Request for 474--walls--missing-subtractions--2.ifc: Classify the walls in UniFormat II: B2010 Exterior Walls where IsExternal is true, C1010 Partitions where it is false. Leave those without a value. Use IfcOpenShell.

First a look at what the model holds.

```python
import ifcopenshell
import ifcopenshell.util.element

model = ifcopenshell.open("474--walls--missing-subtractions--2.ifc")
print(model.schema)
print("classifications:", [c.Name for c in model.by_type("IfcClassification")])
values = [ifcopenshell.util.element.get_pset(e, "Pset_WallCommon", "IsExternal") for e in model.by_type("IfcWall")]
for value in (True, False, None):
    print("IsExternal", value, values.count(value))
```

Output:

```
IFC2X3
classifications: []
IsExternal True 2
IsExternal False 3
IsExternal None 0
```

```python
import ifcopenshell
import ifcopenshell.api.classification
import ifcopenshell.util.element

model = ifcopenshell.open("474--walls--missing-subtractions--2.ifc")

# IFC2X3 requires Source and Edition and has no link from the project to the system.
system = model.create_entity("IfcClassification", Source="ASTM", Edition="E1557", Name="UniFormat II")

walls = model.by_type("IfcWall")
external = {e: ifcopenshell.util.element.get_pset(e, "Pset_WallCommon", "IsExternal") for e in walls}
for flag, code, name in ((True, "B2010", "Exterior Walls"), (False, "C1010", "Partitions")):
    products = [e for e in walls if external[e] is flag]
    ifcopenshell.api.classification.add_reference(
        model, products=products, classification=system, identification=code, name=name
    )
    print(code, len(products))

model.write("474--walls--missing-subtractions--2_rev.ifc")
```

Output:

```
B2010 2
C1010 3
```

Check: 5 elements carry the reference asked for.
